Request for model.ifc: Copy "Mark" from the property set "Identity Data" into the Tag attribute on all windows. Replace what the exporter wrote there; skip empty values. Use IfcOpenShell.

First a look at what the model holds.

```python
import ifcopenshell
import ifcopenshell.util.element

model = ifcopenshell.open("model.ifc")
print(model.schema)
windows = model.by_type("IfcWindow")
print(len(windows), "windows")
for e in windows[:8]:
    source = ifcopenshell.util.element.get_pset(e, "Identity Data", "Mark")
    target = e.Tag
    print(e.id(), repr(source), repr(target), sep=" | ")
```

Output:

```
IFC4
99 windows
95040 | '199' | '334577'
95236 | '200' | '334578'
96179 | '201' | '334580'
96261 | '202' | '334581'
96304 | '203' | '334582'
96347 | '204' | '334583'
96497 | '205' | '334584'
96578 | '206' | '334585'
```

```python
import ifcopenshell
import ifcopenshell.util.element

model = ifcopenshell.open("model.ifc")

count = 0
for e in model.by_type("IfcWindow"):
    value = ifcopenshell.util.element.get_pset(e, "Identity Data", "Mark")
    current = e.Tag
    if not value or not value.strip() or current == value:
        continue
    e.Tag = value
    count += 1

print(count, "windows updated")

model.write("model_v2.ifc")
```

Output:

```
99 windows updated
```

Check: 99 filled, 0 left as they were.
